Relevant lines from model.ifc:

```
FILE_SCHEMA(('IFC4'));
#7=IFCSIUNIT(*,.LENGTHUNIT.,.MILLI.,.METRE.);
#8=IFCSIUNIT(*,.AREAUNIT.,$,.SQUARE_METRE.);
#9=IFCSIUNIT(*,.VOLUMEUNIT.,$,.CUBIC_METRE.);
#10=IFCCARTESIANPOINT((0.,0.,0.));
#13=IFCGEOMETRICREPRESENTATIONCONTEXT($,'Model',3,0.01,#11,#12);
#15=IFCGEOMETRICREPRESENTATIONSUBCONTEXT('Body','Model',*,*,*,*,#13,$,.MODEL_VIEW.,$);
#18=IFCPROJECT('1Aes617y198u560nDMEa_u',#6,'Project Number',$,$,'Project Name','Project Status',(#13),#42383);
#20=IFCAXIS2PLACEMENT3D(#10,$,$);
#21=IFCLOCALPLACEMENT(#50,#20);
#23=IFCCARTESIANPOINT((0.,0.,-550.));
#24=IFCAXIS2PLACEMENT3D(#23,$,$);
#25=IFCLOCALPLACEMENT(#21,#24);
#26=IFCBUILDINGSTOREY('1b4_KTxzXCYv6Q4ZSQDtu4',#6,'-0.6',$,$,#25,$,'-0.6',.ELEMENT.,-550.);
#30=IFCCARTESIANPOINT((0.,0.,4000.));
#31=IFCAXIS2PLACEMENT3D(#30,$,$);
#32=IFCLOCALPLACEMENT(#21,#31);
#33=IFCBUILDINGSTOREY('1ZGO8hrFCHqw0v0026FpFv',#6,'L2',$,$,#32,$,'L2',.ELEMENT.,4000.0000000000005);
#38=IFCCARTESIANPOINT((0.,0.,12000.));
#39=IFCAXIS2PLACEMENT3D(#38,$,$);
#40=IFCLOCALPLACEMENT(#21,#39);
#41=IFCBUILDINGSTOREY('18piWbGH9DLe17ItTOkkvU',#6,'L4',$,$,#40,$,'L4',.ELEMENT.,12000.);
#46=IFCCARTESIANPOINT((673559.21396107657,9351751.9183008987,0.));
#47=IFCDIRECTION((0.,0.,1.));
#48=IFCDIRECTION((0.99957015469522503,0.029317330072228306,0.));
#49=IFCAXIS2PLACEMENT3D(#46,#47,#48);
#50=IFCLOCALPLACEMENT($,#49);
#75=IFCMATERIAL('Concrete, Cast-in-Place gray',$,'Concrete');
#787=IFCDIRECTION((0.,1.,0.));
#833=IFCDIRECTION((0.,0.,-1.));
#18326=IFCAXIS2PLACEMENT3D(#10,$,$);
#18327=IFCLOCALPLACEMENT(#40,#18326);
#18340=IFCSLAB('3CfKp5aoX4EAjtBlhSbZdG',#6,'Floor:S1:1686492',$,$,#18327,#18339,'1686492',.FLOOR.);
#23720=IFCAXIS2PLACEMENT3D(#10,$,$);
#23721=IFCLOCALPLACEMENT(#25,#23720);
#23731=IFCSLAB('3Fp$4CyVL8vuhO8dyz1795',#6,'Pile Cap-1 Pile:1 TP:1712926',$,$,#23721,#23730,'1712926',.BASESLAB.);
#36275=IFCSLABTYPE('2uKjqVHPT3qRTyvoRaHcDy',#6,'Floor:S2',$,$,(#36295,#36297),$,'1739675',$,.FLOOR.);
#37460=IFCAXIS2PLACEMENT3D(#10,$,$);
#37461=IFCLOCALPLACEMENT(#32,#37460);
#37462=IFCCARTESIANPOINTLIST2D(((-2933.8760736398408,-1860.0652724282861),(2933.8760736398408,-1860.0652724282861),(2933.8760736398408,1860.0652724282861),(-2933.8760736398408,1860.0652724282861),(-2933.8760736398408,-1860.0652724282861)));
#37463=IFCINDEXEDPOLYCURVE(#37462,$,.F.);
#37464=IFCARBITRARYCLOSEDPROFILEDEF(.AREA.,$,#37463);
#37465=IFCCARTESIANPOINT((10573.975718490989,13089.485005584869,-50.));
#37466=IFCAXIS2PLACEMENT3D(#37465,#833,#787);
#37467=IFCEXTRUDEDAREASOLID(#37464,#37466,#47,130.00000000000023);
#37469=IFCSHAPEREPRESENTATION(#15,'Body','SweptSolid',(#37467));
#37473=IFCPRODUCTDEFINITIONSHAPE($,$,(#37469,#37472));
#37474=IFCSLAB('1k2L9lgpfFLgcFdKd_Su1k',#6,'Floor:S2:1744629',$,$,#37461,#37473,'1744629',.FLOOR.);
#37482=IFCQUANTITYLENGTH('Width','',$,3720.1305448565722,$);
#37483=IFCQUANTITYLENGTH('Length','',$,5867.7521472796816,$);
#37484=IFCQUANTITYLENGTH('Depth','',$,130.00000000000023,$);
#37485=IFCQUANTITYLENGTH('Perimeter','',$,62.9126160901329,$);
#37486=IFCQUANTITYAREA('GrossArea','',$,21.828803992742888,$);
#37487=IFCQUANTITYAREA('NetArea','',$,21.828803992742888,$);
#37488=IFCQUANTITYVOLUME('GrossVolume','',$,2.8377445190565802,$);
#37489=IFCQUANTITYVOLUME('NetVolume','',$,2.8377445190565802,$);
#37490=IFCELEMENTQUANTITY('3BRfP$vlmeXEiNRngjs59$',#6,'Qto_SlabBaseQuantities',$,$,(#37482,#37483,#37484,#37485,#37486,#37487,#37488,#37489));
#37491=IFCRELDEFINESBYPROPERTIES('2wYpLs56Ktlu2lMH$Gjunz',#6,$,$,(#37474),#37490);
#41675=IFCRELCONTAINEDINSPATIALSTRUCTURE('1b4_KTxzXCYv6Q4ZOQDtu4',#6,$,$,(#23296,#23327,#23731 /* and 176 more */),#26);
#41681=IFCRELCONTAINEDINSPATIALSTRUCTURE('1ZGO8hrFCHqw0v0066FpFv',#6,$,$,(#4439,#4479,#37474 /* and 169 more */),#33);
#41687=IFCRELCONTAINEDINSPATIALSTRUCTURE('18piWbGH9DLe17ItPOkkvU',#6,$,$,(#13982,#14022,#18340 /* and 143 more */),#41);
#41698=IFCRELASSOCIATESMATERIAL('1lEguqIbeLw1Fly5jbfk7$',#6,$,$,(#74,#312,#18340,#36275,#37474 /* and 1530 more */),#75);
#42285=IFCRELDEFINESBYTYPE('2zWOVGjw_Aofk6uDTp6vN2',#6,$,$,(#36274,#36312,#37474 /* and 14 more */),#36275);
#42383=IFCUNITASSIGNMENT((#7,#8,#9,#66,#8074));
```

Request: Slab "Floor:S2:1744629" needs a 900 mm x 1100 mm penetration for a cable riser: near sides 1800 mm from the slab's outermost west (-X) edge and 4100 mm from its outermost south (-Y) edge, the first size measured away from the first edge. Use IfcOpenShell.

```python
import numpy as np
import ifcopenshell
import ifcopenshell.api.feature
import ifcopenshell.api.geometry
import ifcopenshell.api.pset
import ifcopenshell.api.root
import ifcopenshell.geom
import ifcopenshell.util.element
import ifcopenshell.util.placement
import ifcopenshell.util.representation
import ifcopenshell.util.shape
import ifcopenshell.util.unit

model = ifcopenshell.open("model.ifc")
unit_scale = ifcopenshell.util.unit.calculate_unit_scale(model)
area_scale = ifcopenshell.util.unit.calculate_unit_scale(model, "AREAUNIT")
volume_scale = ifcopenshell.util.unit.calculate_unit_scale(model, "VOLUMEUNIT")
settings = ifcopenshell.geom.settings()


def volume(element):
    """Net volume in cubic metres, openings subtracted."""
    shape = ifcopenshell.geom.create_shape(settings, element)
    return ifcopenshell.util.shape.get_volume(shape.geometry)


slab = model.by_id(37474)
before = volume(slab)

# Extent in the slab's own axes, in metres. The edges named are its -X and -Y sides.
slab_shape = ifcopenshell.geom.create_shape(settings, slab)
vertices = ifcopenshell.util.shape.get_vertices(slab_shape.geometry)
x_min, y_min, bottom = vertices.min(axis=0)
top = vertices[:, 2].max()

opening = ifcopenshell.api.root.create_entity(model, ifc_class="IfcOpeningElement", name="Cable riser opening", predefined_type="OPENING")
context = ifcopenshell.util.representation.get_context(model, "Model", "Body", "MODEL_VIEW")
width, depth = 0.9, 1.1
outline = [(0.0, 0.0), (width, 0.0), (width, depth), (0.0, depth), (0.0, 0.0)]
# Overshoot both faces by 50 mm so the cut is clean.
shape = ifcopenshell.api.geometry.add_slab_representation(
    model, context=context, depth=top - bottom + 0.1, polyline=outline
)
ifcopenshell.api.geometry.assign_representation(model, product=opening, representation=shape)

matrix = ifcopenshell.util.placement.get_local_placement(slab.ObjectPlacement)
matrix[:, 3] = matrix @ np.append(np.array([x_min + 1.8, y_min + 4.1, bottom - 0.05]) / unit_scale, 1.0)
ifcopenshell.api.geometry.edit_object_placement(model, product=opening, matrix=matrix, is_si=False)
ifcopenshell.api.feature.add_feature(model, feature=opening, element=slab)

after = volume(slab)

# Update the slab's stored quantities.
qto = model.by_id(ifcopenshell.util.element.get_pset(slab, "Qto_SlabBaseQuantities", should_inherit=False)["id"])
ifcopenshell.api.pset.edit_qto(model, qto=qto, properties={
    "NetArea": after / (top - bottom) / area_scale,
    "NetVolume": after / volume_scale,
})

print(f"slab volume {before:.3f} -> {after:.3f} m3")

model.write("model_updated.ifc")
```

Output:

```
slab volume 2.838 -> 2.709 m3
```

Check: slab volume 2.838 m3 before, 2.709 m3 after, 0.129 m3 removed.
